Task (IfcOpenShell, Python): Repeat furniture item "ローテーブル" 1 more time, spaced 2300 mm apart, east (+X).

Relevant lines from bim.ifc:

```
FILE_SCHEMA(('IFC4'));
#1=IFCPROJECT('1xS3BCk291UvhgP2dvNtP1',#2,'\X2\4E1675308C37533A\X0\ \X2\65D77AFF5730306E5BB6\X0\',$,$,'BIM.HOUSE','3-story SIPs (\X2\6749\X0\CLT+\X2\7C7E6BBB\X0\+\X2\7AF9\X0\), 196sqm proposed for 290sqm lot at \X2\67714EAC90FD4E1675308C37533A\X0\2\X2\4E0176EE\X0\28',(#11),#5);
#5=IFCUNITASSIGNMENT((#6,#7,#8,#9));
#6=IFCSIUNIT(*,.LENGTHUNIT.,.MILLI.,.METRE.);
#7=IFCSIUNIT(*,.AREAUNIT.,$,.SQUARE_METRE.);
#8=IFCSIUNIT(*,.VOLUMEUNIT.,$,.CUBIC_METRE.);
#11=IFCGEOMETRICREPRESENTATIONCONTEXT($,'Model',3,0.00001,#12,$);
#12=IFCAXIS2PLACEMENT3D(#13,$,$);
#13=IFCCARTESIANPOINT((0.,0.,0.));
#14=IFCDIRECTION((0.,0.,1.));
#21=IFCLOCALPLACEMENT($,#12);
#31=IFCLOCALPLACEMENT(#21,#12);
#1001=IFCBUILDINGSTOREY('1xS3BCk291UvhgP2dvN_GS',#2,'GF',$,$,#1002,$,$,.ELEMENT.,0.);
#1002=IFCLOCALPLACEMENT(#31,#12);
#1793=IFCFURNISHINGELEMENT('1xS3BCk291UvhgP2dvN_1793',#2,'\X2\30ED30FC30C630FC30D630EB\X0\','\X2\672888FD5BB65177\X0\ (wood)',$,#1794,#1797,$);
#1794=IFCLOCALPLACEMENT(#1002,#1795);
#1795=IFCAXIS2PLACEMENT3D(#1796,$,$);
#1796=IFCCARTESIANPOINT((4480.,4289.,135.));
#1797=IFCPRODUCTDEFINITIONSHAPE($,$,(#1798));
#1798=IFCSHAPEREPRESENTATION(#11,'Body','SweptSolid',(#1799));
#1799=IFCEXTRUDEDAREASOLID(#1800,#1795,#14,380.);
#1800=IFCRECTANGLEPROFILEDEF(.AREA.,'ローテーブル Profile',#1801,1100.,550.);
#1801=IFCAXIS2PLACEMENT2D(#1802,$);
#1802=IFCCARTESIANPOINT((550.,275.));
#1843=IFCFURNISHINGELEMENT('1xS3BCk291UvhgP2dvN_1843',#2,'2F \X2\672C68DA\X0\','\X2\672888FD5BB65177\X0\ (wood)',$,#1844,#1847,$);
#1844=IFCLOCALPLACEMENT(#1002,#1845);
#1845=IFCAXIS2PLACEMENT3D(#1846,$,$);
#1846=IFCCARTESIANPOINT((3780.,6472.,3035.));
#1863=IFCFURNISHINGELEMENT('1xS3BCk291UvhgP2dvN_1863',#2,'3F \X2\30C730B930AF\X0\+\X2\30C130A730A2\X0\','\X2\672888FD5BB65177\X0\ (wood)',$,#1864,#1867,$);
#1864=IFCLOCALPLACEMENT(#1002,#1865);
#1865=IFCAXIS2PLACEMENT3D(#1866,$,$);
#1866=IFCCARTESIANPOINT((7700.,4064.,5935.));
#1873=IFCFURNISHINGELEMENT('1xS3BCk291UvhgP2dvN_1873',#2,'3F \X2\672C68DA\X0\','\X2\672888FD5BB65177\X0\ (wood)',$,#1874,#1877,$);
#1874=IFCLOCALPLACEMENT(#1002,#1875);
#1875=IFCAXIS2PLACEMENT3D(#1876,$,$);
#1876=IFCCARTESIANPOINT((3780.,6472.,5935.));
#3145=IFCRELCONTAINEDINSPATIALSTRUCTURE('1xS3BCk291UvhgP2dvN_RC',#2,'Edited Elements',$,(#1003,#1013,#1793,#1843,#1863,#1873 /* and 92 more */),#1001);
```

```python
import numpy as np
import ifcopenshell
import ifcopenshell.api.geometry
import ifcopenshell.api.root
import ifcopenshell.util.element
import ifcopenshell.util.placement

model = ifcopenshell.open("bim.ifc")


def reuse_history(source, copy):
    """copy_class also copies each property set's owner history, people and application; keep the originals."""
    for rel in copy.IsDefinedBy:
        if rel.is_a("IfcRelDefinesByProperties") and (history := rel.RelatingPropertyDefinition.OwnerHistory):
            rel.RelatingPropertyDefinition.OwnerHistory = source.OwnerHistory
            ifcopenshell.util.element.remove_deep2(model, history)


source = model.by_guid("1xS3BCk291UvhgP2dvN_1793")
base = ifcopenshell.util.placement.get_local_placement(source.ObjectPlacement)
step = np.array([1.0, 0.0, 0.0]) * 2300.0

for i in range(1, 2):
    copy = ifcopenshell.api.root.copy_class(model, product=source)
    copy.Representation = ifcopenshell.util.element.copy_deep(
        model, source.Representation, exclude=["IfcGeometricRepresentationContext", "IfcRepresentationMap"]
    )
    reuse_history(source, copy)
    matrix = base.copy()
    matrix[:3, 3] += i * step
    print("added at", matrix[:3, 3].round(3) + 0.0)
    ifcopenshell.api.geometry.edit_object_placement(model, product=copy, matrix=matrix, is_si=False)

model.write("bim_updated.ifc")
```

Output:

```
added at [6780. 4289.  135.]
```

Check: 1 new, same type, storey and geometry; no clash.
